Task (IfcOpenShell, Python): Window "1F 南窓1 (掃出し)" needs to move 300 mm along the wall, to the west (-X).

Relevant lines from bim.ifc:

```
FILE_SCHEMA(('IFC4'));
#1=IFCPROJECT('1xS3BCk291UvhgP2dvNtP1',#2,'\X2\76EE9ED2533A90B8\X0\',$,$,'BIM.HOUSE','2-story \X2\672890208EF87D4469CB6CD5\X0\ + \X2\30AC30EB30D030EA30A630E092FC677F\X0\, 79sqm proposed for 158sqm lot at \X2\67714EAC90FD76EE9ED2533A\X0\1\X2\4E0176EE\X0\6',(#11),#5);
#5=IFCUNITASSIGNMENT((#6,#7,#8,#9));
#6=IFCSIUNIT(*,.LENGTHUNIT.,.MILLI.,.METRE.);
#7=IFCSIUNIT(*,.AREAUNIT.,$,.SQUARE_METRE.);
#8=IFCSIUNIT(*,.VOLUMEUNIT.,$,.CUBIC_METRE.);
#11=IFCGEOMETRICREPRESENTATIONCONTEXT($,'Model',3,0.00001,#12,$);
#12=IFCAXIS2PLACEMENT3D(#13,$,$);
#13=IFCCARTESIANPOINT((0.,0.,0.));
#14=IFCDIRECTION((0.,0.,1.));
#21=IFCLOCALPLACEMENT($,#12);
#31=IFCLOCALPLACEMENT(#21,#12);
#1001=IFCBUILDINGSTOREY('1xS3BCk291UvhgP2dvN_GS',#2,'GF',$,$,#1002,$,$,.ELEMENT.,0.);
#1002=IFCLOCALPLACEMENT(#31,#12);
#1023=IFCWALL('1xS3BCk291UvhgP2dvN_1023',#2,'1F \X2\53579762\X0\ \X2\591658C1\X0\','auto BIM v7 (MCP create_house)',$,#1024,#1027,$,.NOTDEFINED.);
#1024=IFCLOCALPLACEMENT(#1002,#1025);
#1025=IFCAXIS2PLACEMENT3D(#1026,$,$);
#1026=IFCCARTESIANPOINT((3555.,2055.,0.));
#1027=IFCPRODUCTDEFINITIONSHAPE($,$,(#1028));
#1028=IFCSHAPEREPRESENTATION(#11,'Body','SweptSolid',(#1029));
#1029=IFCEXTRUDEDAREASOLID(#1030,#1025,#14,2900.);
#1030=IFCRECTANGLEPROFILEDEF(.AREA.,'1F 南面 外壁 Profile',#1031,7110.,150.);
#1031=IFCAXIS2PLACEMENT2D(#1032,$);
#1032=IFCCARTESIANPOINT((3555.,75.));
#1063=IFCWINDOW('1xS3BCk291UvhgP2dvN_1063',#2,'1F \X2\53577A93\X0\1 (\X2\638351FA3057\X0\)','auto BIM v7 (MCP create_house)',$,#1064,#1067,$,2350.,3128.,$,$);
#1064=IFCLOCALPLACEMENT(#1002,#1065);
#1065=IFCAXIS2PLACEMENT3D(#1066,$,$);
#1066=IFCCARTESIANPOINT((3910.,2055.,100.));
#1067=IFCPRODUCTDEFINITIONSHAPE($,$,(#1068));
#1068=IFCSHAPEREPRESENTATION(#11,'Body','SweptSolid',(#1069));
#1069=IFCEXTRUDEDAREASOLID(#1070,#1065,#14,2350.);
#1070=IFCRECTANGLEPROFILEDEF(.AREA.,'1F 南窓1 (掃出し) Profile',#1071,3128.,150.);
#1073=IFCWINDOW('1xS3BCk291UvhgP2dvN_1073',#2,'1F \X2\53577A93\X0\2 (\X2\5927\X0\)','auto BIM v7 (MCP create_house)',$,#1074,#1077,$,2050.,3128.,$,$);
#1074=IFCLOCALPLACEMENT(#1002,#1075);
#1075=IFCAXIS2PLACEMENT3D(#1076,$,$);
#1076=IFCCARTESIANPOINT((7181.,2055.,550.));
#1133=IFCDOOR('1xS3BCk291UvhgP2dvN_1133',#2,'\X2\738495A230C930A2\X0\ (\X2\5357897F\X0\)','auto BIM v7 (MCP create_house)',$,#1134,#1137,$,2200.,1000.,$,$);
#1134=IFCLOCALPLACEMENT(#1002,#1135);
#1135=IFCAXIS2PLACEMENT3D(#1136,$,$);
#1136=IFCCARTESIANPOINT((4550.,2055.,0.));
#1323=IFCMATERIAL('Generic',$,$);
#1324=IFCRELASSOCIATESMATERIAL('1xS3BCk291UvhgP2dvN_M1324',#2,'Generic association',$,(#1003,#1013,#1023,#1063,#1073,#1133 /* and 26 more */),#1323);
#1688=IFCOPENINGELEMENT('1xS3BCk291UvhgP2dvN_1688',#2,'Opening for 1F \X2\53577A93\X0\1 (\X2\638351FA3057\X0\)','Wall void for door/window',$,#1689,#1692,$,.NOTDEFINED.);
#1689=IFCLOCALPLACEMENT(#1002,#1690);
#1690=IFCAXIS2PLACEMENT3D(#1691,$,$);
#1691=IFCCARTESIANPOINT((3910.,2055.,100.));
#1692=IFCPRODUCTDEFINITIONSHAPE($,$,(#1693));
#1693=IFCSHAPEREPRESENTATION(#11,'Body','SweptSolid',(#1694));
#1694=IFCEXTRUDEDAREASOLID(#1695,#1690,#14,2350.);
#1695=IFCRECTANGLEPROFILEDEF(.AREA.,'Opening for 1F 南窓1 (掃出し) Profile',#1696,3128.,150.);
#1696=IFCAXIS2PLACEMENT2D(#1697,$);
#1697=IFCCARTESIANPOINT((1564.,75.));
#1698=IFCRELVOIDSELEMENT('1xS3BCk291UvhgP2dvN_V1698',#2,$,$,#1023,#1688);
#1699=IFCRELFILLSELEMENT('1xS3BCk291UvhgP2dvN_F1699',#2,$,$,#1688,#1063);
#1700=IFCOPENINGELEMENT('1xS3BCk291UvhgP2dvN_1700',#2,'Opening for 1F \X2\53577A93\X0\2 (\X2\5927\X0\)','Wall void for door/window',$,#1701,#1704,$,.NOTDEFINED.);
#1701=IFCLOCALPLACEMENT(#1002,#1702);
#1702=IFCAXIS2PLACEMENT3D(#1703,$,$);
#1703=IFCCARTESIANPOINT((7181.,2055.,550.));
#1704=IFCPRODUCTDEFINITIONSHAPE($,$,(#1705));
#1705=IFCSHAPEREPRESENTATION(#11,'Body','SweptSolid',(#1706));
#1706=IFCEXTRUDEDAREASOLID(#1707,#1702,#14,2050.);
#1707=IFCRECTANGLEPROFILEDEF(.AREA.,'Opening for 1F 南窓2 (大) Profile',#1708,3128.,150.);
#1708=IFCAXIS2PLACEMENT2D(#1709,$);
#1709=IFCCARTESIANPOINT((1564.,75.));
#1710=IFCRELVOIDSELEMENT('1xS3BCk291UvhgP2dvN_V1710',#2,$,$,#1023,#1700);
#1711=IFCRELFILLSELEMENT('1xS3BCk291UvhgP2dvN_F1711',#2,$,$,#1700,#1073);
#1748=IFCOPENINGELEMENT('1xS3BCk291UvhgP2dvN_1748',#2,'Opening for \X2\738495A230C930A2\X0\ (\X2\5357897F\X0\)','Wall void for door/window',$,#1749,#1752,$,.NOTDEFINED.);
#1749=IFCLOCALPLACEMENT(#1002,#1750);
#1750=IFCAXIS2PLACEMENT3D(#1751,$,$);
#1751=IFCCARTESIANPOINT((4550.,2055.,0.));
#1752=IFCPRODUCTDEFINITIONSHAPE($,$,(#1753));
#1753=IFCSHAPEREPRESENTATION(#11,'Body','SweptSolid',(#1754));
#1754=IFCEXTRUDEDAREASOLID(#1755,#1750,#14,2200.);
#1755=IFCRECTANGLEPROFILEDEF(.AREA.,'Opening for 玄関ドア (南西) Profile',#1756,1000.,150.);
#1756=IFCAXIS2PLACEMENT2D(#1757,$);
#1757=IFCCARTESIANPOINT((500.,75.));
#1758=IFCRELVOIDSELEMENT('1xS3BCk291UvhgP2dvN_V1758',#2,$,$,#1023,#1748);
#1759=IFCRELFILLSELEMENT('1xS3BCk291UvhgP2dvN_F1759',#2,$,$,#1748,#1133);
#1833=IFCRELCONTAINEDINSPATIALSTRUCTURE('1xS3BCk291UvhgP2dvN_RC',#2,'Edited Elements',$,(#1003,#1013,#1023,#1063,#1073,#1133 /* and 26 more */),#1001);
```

```python
import ifcopenshell
import ifcopenshell.api.geometry
import ifcopenshell.util.placement
import ifcopenshell.util.unit

model = ifcopenshell.open("bim.ifc")
unit_scale = ifcopenshell.util.unit.calculate_unit_scale(model)

window = model.by_guid("1xS3BCk291UvhgP2dvN_1063")
opening = window.FillsVoids[0].RelatingOpeningElement
wall = opening.VoidsElements[0].RelatingBuildingElement

wall_matrix = ifcopenshell.util.placement.get_local_placement(wall.ObjectPlacement)
shift = wall_matrix[:3, 0] * -0.3 / unit_scale
before = ifcopenshell.util.placement.get_local_placement(window.ObjectPlacement)[:3, 3].copy()

# The window is not placed relative to its opening, so move both.
for product in (opening, window):
    matrix = ifcopenshell.util.placement.get_local_placement(product.ObjectPlacement)
    matrix[:3, 3] += shift
    ifcopenshell.api.geometry.edit_object_placement(model, product=product, matrix=matrix, is_si=False)

after = ifcopenshell.util.placement.get_local_placement(window.ObjectPlacement)[:3, 3]
print("window moved by", (after - before).round(3) + 0.0)

model.write("bim_edited.ifc")
```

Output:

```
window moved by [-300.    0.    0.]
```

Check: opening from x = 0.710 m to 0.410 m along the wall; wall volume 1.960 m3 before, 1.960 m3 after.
